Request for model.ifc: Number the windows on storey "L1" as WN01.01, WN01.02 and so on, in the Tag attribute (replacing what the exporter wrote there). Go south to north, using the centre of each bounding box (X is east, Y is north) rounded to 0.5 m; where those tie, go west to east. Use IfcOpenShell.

First a look at what the model holds.

```python
import ifcopenshell
import ifcopenshell.util.element
import ifcopenshell.util.placement

model = ifcopenshell.open("model.ifc")
print(model.schema)
storey = next(s for s in model.by_type("IfcBuildingStorey") if s.Name == "L1")
windows = [e for e in ifcopenshell.util.element.get_decomposition(storey) if e.is_a("IfcWindow")]
for e in sorted(windows, key=lambda e: e.id()):
    origin = ifcopenshell.util.placement.get_local_placement(e.ObjectPlacement)[:3, 3]
    print(e.id(), e.Tag, e.Name, origin.round(2) + 0.0, sep=" | ")
```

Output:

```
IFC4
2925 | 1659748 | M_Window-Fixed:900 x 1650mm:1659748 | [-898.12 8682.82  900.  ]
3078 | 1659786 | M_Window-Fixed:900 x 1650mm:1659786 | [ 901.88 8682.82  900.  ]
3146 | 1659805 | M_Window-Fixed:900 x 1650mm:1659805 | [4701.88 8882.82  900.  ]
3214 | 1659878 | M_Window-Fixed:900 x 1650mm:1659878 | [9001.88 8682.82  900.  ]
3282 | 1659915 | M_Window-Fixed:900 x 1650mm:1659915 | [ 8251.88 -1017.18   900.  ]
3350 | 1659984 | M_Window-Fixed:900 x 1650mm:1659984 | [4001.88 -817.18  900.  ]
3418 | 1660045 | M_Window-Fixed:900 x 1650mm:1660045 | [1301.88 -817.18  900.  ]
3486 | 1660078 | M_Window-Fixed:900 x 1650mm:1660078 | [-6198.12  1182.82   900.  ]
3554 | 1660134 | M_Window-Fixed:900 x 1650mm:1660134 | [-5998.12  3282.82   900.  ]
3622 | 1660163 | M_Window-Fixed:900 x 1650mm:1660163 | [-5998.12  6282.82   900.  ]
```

```python
import ifcopenshell
import ifcopenshell.geom
import ifcopenshell.util.element
import ifcopenshell.util.shape

model = ifcopenshell.open("model.ifc")
settings = ifcopenshell.geom.settings()
settings.set("use-world-coords", True)


def centre(element):
    shape = ifcopenshell.geom.create_shape(settings, element)
    return ifcopenshell.util.shape.get_bbox_centroid(shape.geometry)


storey = next(s for s in model.by_type("IfcBuildingStorey") if s.Name == "L1")
windows = [e for e in ifcopenshell.util.element.get_decomposition(storey) if e.is_a("IfcWindow")]

# Insertion points can sit at a corner or the storey origin, so sort by the geometry (in metres).
centres = {e: centre(e) for e in windows}
windows.sort(key=lambda e: (round(centres[e][1] / 0.5), centres[e][0]))

for i, e in enumerate(windows, start=1):
    number = f"WN01.{i:02d}"
    e.Tag = number
    print(e.id(), number)

model.write("model_updated.ifc")
```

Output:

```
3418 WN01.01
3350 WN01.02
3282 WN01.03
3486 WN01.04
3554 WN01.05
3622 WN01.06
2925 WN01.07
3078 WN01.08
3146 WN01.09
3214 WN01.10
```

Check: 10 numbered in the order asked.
